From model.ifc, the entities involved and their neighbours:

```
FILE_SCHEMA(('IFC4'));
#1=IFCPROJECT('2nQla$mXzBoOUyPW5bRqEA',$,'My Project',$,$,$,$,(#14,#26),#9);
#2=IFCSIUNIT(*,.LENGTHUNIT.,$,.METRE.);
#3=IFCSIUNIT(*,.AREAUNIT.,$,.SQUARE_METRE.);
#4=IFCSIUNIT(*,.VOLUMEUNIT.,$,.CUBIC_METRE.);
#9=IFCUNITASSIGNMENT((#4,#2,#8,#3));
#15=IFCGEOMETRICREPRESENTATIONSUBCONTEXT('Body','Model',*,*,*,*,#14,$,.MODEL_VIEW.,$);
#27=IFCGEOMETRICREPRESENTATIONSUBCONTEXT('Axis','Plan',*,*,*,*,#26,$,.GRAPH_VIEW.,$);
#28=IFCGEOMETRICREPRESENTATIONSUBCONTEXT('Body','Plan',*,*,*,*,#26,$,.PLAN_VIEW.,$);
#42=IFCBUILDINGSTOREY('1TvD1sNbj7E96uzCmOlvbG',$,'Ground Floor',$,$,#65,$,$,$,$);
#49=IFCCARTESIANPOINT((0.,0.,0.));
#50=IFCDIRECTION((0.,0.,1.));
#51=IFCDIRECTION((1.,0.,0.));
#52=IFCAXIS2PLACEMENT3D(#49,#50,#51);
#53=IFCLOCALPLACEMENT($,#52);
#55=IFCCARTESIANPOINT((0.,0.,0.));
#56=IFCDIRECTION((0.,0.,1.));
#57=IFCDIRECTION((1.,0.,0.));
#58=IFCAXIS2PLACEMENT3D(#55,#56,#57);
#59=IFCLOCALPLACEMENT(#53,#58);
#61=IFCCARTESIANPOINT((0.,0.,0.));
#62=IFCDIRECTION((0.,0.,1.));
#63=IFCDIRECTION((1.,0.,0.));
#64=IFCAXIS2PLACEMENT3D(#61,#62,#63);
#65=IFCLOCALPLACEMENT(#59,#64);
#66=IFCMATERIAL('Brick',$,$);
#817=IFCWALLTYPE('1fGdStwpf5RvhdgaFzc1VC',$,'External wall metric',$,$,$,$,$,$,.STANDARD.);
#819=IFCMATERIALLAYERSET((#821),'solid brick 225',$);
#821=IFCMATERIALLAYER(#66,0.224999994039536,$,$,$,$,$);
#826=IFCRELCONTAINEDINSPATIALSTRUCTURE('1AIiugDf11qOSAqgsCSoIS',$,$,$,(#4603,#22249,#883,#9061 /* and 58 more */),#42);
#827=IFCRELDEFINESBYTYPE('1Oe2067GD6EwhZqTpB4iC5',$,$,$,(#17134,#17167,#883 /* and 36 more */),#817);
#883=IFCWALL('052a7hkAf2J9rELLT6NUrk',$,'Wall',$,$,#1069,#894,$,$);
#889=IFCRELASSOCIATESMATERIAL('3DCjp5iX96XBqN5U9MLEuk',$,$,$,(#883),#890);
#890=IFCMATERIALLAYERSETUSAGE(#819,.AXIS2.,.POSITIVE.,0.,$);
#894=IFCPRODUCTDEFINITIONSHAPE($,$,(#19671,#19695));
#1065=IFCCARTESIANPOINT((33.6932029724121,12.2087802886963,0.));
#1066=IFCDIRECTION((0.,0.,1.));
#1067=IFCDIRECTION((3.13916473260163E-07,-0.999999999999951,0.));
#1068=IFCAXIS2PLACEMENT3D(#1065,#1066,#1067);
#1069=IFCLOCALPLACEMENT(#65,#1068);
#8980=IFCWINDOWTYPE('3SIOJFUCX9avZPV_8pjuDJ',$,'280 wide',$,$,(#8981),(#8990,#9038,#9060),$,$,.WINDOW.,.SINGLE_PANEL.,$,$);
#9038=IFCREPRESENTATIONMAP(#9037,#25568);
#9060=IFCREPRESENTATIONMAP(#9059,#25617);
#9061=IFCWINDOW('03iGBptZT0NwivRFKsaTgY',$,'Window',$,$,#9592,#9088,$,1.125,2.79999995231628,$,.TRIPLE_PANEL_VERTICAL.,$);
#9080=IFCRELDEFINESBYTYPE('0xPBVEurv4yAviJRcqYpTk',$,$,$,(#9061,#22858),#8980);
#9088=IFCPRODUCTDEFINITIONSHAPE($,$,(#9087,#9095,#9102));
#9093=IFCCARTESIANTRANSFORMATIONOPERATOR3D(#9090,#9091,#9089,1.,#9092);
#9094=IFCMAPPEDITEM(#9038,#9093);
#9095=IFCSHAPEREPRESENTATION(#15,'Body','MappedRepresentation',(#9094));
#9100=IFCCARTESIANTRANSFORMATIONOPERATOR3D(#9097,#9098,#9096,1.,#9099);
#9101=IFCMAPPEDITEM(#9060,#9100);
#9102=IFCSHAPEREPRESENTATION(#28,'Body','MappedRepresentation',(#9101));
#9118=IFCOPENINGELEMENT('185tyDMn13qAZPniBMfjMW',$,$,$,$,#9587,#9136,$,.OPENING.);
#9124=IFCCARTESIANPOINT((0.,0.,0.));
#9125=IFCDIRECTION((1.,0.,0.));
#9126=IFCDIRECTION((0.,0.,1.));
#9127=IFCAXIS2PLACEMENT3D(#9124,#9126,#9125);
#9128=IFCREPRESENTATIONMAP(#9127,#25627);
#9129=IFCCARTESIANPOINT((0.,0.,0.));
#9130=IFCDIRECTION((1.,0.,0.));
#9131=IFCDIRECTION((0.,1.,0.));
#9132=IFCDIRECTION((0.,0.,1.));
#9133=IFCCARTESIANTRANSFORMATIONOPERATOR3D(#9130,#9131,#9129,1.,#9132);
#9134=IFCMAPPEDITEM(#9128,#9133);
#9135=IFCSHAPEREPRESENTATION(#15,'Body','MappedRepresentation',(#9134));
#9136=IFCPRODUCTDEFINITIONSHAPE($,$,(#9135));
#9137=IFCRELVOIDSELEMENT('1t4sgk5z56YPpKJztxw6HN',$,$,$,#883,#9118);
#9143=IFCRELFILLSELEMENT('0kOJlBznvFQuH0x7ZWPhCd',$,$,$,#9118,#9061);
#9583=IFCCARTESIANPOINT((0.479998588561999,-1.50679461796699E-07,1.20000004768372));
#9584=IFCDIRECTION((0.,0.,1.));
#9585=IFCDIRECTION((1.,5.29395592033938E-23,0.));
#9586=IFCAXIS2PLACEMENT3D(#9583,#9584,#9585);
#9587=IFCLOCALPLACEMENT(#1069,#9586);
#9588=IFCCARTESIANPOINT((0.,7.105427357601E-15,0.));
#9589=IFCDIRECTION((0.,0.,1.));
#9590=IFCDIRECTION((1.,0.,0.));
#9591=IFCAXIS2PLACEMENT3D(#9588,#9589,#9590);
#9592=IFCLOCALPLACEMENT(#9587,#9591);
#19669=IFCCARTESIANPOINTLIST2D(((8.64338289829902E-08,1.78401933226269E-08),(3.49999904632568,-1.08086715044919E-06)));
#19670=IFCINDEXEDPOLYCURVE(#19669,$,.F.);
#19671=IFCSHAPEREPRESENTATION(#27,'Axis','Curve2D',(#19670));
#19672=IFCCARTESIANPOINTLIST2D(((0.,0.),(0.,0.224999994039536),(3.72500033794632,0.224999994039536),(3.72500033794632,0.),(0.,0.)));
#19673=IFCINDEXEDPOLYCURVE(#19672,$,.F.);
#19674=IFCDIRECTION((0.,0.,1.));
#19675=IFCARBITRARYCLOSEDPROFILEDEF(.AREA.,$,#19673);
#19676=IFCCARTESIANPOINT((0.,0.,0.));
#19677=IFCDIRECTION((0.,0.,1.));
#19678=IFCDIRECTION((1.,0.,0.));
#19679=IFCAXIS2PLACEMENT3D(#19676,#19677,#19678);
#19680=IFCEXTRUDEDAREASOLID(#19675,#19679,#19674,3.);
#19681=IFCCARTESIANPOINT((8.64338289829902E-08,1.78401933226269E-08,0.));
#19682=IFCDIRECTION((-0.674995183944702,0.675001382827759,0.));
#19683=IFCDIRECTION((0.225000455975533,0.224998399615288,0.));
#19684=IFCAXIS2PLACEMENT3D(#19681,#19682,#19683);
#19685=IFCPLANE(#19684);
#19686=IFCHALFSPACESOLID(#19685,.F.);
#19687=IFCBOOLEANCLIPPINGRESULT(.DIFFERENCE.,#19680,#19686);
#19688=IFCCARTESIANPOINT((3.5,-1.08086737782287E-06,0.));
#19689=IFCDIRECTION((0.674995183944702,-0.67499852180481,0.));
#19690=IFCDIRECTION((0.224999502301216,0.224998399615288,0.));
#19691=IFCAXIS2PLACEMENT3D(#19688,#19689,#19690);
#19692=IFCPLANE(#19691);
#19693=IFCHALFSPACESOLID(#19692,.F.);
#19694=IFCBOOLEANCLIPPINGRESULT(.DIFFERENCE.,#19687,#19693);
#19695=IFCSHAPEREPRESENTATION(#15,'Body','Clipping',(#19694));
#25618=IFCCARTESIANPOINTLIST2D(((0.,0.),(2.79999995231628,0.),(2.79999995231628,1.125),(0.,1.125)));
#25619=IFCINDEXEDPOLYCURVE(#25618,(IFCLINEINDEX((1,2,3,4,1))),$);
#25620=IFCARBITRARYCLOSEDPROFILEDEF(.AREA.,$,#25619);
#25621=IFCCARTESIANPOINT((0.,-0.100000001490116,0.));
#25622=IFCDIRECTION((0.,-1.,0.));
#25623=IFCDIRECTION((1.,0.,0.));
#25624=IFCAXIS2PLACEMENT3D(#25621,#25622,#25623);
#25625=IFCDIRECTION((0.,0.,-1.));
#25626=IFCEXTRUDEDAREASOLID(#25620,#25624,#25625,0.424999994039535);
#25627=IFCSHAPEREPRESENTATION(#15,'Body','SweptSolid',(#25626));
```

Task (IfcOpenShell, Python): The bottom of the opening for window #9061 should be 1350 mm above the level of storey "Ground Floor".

```python
import numpy as np
import ifcopenshell
import ifcopenshell.api.geometry
import ifcopenshell.geom
import ifcopenshell.util.element
import ifcopenshell.util.placement
import ifcopenshell.util.shape
import ifcopenshell.util.unit

model = ifcopenshell.open("model.ifc")
unit_scale = ifcopenshell.util.unit.calculate_unit_scale(model)

window = model.by_id(9061)
opening = window.FillsVoids[0].RelatingOpeningElement
storey = ifcopenshell.util.element.get_container(window, ifc_class="IfcBuildingStorey")
level = ifcopenshell.util.placement.get_local_placement(storey.ObjectPlacement)[2, 3]

# The opening's origin need not be at the sill, so measure its lowest point.
shape = ifcopenshell.geom.create_shape(ifcopenshell.geom.settings(), opening)
bottom = ifcopenshell.util.shape.get_shape_bottom_elevation(shape, shape.geometry) / unit_scale
dz = level + 1.35 / unit_scale - bottom

shift = np.array([0.0, 0.0, dz])
# The window is placed relative to its opening, so it follows when the opening moves.
matrix = ifcopenshell.util.placement.get_local_placement(opening.ObjectPlacement)
matrix[:3, 3] += shift
ifcopenshell.api.geometry.edit_object_placement(
    model, product=opening, matrix=matrix, is_si=False, should_transform_children=True
)

print(f"moved by {dz * unit_scale:+.3f} m")

model.write("model_rev.ifc")
```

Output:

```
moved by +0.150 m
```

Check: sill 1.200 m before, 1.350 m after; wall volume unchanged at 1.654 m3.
